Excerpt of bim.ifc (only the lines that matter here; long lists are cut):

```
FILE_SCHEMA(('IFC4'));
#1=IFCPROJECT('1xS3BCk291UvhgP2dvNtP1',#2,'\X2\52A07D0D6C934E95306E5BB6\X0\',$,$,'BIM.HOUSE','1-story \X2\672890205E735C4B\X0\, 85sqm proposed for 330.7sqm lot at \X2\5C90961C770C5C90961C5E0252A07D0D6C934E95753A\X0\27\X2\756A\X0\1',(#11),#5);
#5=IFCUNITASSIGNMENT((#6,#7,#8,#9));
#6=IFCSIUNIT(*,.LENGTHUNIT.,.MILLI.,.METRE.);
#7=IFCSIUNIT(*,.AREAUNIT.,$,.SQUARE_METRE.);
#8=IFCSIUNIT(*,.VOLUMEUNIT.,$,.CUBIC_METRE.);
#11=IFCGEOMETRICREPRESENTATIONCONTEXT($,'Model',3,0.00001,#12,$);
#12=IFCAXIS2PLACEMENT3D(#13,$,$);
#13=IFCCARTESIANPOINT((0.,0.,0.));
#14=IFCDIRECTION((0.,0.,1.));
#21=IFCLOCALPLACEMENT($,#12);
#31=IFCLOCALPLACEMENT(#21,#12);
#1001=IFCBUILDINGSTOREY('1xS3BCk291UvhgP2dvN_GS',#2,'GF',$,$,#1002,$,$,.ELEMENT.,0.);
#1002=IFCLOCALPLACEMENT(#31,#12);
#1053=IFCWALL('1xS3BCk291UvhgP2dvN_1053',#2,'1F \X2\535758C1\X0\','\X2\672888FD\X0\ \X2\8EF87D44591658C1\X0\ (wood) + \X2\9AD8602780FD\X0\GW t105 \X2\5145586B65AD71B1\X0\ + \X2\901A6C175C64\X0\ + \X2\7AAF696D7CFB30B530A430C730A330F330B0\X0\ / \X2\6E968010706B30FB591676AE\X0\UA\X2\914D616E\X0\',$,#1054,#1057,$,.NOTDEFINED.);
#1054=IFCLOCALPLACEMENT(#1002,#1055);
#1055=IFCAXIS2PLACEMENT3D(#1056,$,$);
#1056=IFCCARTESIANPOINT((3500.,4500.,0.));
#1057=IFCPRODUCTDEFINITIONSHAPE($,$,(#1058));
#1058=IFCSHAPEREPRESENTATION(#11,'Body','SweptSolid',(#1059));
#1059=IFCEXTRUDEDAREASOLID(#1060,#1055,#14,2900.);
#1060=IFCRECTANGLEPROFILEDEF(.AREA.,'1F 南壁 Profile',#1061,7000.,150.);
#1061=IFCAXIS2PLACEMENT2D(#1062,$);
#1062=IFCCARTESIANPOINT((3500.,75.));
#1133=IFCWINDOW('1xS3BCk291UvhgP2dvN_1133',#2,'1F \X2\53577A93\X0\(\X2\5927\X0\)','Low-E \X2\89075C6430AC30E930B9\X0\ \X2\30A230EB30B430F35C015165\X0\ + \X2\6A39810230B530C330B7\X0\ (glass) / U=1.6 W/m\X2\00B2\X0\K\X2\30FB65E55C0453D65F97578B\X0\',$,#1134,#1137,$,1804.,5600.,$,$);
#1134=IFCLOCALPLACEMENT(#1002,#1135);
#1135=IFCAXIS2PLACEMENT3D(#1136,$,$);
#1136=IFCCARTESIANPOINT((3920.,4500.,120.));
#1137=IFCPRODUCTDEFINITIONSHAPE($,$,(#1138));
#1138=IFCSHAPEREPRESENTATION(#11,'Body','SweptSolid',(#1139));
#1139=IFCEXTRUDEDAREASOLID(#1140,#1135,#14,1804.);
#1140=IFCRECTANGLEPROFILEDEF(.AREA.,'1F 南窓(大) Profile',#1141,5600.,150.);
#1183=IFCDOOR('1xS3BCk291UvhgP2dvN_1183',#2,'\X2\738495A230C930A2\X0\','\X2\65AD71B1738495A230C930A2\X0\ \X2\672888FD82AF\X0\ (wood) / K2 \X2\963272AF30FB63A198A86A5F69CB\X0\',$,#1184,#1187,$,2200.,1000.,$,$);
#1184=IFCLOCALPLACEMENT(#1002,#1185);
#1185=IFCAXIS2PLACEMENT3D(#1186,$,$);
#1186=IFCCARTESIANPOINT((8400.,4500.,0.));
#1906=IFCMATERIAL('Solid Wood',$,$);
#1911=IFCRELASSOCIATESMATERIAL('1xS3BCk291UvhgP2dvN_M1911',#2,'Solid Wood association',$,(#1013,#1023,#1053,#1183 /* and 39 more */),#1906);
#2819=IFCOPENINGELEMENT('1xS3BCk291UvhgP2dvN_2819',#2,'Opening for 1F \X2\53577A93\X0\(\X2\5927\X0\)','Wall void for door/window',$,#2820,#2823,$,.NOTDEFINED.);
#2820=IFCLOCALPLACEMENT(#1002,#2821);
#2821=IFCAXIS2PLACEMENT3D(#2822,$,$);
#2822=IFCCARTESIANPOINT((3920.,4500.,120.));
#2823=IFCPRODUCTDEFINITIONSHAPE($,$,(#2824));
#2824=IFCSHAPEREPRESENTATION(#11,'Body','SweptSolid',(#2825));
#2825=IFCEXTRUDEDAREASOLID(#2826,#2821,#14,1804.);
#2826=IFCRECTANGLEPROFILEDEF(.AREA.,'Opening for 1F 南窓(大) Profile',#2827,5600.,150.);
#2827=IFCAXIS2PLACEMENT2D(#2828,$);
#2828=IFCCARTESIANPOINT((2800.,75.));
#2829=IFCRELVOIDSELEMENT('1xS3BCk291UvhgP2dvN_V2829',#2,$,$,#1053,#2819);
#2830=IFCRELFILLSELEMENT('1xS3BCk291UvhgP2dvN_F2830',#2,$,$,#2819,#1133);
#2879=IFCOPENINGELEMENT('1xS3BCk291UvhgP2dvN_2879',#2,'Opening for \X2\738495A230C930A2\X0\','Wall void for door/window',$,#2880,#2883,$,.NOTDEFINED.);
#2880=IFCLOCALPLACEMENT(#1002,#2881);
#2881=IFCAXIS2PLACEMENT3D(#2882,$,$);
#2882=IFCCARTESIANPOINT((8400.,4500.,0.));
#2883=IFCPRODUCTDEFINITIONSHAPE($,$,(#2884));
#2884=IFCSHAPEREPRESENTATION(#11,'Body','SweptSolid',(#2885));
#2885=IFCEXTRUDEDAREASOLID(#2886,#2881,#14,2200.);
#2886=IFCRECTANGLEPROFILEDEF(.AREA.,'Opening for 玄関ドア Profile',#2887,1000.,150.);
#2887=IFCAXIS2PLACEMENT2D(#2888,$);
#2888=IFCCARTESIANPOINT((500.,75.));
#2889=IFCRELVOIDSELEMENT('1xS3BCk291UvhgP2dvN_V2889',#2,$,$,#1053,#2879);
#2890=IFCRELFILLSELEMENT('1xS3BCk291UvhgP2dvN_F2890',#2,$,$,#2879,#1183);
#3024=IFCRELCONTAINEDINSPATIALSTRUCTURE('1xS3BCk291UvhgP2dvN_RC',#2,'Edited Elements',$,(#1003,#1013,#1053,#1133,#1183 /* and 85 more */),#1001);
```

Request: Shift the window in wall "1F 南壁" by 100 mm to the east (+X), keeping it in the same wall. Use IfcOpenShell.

```python
import ifcopenshell
import ifcopenshell.api.geometry
import ifcopenshell.util.placement

model = ifcopenshell.open("bim.ifc")

window = model.by_id(1133)
opening = window.FillsVoids[0].RelatingOpeningElement
wall = opening.VoidsElements[0].RelatingBuildingElement

wall_matrix = ifcopenshell.util.placement.get_local_placement(wall.ObjectPlacement)
shift = wall_matrix[:3, 0] * 100.0
before = ifcopenshell.util.placement.get_local_placement(window.ObjectPlacement)[:3, 3].copy()

# The window is not placed relative to its opening, so move both.
for product in (opening, window):
    matrix = ifcopenshell.util.placement.get_local_placement(product.ObjectPlacement)
    matrix[:3, 3] += shift
    ifcopenshell.api.geometry.edit_object_placement(model, product=product, matrix=matrix, is_si=False)

after = ifcopenshell.util.placement.get_local_placement(window.ObjectPlacement)[:3, 3]
print("window moved by", (after - before).round(3) + 0.0)

model.write("bim_edited.ifc")
```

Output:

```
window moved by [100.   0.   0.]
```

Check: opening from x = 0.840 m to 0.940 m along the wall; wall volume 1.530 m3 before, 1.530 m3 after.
